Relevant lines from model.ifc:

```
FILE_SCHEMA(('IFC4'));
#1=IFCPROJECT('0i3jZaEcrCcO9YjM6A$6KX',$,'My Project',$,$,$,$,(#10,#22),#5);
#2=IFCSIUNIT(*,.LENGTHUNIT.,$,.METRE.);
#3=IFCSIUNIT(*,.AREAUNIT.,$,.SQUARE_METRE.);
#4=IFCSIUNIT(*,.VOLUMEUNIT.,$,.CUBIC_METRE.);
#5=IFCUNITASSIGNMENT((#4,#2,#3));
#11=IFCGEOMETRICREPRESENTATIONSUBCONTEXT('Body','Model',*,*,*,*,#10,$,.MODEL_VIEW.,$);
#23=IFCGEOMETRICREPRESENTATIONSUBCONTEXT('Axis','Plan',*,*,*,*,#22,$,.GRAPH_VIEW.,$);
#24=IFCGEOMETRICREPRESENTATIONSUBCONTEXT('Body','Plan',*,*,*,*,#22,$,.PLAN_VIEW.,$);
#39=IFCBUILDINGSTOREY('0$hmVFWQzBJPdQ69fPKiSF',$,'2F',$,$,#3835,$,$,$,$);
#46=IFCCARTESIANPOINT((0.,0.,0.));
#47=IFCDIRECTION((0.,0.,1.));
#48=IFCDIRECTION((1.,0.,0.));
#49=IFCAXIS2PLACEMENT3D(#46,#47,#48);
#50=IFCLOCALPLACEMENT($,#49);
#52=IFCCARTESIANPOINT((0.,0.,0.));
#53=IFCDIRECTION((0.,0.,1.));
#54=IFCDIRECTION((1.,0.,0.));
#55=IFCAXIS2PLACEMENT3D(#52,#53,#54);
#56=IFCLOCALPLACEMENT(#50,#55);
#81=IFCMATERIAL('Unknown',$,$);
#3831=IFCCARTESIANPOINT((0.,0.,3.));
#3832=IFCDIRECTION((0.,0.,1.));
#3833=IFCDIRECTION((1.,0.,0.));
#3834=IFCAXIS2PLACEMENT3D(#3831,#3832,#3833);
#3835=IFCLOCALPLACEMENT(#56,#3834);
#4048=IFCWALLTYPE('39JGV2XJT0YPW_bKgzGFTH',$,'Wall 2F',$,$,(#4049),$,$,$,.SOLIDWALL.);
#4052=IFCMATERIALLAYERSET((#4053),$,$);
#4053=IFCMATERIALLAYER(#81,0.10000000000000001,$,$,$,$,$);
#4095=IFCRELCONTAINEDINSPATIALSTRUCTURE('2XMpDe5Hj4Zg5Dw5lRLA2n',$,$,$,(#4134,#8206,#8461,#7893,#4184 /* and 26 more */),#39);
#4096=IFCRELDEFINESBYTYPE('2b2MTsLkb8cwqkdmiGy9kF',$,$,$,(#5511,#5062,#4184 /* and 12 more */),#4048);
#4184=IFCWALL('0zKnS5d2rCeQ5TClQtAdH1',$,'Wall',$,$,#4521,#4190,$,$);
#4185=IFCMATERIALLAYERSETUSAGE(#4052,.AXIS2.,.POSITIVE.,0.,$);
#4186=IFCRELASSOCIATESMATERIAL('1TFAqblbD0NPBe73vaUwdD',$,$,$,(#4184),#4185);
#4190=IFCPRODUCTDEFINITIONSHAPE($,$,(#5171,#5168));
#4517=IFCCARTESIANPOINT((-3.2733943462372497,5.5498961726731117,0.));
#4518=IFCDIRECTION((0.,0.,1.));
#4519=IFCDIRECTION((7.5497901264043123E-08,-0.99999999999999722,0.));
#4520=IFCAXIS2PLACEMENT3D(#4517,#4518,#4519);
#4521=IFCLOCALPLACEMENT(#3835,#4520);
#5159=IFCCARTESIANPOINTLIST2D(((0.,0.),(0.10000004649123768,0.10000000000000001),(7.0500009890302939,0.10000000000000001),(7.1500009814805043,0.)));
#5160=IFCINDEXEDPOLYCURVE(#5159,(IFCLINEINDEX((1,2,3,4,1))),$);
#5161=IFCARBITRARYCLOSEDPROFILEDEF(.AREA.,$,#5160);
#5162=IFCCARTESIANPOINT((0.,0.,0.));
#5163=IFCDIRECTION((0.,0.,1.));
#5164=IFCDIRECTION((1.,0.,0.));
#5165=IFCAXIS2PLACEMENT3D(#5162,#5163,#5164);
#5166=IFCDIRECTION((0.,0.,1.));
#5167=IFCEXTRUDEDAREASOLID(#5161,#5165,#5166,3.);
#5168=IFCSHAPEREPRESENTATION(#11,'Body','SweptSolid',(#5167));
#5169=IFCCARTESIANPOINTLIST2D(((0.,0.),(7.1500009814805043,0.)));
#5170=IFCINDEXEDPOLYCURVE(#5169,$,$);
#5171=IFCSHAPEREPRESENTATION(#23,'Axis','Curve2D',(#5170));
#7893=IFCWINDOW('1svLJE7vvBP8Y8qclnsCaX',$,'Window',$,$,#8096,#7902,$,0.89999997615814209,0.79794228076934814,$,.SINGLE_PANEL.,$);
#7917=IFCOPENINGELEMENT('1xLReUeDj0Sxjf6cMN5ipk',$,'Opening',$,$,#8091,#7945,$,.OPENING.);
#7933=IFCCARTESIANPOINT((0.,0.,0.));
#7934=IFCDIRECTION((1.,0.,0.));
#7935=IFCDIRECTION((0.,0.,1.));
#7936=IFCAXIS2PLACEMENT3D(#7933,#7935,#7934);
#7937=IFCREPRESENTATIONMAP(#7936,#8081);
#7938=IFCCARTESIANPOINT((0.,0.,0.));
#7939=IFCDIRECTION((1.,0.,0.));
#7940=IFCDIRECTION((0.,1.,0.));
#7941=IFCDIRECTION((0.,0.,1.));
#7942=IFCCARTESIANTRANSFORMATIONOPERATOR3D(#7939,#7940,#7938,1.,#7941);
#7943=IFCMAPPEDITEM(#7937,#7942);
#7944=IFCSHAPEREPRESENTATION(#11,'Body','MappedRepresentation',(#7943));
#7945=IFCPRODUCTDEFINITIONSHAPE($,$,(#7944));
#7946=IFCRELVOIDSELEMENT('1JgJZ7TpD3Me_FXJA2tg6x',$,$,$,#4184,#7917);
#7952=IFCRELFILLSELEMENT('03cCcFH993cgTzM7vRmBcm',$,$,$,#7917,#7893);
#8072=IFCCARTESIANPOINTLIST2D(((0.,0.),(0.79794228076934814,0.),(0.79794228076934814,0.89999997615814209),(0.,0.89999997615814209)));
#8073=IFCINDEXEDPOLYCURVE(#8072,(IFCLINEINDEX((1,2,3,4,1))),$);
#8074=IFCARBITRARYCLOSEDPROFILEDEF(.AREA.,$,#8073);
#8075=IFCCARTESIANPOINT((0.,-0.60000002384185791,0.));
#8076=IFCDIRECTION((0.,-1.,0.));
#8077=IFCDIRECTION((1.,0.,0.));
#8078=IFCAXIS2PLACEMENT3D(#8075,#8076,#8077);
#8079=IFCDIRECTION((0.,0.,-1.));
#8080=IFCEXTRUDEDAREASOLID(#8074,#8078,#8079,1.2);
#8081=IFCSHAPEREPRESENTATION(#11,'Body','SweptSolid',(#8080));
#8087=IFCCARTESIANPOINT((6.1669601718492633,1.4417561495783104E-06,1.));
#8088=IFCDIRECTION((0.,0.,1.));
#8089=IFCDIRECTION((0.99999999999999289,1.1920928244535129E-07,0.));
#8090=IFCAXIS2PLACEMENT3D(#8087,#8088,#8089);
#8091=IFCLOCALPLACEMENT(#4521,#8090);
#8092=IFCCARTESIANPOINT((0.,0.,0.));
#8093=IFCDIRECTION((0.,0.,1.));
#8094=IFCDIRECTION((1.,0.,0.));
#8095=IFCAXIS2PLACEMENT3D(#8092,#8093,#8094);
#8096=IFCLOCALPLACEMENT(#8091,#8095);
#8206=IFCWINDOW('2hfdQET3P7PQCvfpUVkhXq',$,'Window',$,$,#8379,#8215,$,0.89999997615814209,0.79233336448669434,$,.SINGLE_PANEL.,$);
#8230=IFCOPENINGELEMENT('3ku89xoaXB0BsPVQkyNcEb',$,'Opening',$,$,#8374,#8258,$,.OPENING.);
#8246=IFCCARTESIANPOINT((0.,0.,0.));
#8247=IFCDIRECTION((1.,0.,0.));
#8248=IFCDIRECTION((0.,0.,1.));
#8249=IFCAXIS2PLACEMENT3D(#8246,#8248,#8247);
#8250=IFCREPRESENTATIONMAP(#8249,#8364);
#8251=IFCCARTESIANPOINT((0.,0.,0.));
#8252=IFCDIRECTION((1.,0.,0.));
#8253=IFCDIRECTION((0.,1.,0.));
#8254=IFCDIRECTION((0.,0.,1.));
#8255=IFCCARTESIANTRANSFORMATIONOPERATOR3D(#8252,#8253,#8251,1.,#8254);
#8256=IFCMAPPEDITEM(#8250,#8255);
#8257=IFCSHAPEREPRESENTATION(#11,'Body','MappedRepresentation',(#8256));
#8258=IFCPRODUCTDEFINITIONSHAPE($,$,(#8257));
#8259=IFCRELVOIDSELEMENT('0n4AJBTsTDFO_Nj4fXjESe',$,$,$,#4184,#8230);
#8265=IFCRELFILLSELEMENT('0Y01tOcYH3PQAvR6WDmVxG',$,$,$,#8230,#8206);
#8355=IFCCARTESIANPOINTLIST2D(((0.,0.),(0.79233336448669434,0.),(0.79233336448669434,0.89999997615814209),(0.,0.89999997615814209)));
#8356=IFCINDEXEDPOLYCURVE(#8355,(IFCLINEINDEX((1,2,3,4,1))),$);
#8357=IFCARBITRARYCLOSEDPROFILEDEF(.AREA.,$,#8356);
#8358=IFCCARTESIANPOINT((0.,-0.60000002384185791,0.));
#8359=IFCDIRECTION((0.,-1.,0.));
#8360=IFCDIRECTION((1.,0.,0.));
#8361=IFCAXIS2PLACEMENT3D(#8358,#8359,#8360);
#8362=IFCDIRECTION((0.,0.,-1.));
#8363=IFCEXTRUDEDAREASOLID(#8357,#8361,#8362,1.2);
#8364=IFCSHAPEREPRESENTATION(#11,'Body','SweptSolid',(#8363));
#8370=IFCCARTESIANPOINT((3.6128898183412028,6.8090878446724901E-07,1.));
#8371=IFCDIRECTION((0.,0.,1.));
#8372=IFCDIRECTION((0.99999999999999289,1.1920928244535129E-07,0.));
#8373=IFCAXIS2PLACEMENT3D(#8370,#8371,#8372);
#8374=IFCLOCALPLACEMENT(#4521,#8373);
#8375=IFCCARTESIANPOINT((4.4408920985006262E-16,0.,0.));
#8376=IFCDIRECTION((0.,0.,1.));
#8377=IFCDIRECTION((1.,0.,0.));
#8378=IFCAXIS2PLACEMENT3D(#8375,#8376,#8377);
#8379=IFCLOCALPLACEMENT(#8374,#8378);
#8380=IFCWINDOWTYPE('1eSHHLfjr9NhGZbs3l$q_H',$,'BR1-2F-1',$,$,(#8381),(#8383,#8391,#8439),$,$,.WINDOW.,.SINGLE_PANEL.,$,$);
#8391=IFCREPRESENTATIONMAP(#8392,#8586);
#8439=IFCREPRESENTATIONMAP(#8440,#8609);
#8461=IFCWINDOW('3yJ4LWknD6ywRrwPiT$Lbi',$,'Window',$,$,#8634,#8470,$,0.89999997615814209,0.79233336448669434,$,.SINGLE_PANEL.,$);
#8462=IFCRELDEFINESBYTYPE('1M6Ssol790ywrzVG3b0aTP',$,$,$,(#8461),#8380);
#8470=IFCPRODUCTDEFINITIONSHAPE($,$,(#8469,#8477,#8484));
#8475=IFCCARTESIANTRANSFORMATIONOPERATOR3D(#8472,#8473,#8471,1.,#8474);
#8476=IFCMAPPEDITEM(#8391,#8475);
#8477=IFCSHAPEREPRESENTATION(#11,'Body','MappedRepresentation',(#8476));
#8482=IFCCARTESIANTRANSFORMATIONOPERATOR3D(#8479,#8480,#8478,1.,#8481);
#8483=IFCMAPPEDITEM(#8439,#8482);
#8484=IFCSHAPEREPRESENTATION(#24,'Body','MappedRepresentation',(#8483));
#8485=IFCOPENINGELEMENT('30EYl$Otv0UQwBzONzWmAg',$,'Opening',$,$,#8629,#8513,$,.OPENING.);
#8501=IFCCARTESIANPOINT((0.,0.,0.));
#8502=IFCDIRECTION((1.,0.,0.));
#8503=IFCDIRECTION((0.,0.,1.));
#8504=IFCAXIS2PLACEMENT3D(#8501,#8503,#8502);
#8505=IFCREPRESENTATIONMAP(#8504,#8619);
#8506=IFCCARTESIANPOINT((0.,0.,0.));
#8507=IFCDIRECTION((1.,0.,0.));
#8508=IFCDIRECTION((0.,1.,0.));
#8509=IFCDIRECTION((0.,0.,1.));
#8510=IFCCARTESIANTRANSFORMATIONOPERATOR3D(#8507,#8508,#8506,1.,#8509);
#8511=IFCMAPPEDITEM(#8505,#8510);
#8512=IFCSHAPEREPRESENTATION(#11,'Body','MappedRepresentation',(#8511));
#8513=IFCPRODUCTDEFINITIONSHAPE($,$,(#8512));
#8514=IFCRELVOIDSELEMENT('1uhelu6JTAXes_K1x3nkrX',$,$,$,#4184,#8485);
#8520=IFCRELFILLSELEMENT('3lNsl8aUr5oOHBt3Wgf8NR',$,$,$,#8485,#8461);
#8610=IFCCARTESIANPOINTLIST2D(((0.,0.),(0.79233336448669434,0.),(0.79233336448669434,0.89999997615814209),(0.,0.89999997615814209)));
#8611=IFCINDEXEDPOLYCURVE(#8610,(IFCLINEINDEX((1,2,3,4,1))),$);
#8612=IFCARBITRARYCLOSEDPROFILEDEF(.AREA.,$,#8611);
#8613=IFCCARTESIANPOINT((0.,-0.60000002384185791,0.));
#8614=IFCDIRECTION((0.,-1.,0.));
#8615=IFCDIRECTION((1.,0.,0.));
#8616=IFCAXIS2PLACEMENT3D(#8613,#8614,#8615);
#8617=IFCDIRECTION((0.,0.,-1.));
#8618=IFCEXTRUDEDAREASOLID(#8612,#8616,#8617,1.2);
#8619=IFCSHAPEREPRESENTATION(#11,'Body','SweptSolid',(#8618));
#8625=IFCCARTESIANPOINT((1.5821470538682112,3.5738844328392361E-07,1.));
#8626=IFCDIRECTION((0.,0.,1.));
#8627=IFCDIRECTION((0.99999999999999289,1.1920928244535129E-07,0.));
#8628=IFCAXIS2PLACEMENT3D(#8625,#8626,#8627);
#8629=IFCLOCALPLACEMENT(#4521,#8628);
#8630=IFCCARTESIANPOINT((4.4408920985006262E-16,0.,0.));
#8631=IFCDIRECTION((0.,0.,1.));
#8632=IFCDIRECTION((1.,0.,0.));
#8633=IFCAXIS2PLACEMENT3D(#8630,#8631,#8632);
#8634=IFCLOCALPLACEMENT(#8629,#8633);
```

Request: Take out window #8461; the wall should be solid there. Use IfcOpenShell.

```python
import ifcopenshell
import ifcopenshell.api.feature
import ifcopenshell.api.root
import ifcopenshell.geom
import ifcopenshell.util.shape

model = ifcopenshell.open("model.ifc")
settings = ifcopenshell.geom.settings()


def volume(element):
    """Net volume in cubic metres, openings subtracted."""
    shape = ifcopenshell.geom.create_shape(settings, element)
    return ifcopenshell.util.shape.get_volume(shape.geometry)


window = model.by_id(8461)
opening = window.FillsVoids[0].RelatingOpeningElement
wall = opening.VoidsElements[0].RelatingBuildingElement
before = volume(wall)

ifcopenshell.api.root.remove_product(model, product=window)
ifcopenshell.api.feature.remove_feature(model, feature=opening)

after = volume(wall)

print(f"wall volume {before:.3f} -> {after:.3f} m3")

model.write("model_rev.ifc")
```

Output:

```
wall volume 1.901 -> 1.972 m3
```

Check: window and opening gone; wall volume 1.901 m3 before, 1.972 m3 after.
